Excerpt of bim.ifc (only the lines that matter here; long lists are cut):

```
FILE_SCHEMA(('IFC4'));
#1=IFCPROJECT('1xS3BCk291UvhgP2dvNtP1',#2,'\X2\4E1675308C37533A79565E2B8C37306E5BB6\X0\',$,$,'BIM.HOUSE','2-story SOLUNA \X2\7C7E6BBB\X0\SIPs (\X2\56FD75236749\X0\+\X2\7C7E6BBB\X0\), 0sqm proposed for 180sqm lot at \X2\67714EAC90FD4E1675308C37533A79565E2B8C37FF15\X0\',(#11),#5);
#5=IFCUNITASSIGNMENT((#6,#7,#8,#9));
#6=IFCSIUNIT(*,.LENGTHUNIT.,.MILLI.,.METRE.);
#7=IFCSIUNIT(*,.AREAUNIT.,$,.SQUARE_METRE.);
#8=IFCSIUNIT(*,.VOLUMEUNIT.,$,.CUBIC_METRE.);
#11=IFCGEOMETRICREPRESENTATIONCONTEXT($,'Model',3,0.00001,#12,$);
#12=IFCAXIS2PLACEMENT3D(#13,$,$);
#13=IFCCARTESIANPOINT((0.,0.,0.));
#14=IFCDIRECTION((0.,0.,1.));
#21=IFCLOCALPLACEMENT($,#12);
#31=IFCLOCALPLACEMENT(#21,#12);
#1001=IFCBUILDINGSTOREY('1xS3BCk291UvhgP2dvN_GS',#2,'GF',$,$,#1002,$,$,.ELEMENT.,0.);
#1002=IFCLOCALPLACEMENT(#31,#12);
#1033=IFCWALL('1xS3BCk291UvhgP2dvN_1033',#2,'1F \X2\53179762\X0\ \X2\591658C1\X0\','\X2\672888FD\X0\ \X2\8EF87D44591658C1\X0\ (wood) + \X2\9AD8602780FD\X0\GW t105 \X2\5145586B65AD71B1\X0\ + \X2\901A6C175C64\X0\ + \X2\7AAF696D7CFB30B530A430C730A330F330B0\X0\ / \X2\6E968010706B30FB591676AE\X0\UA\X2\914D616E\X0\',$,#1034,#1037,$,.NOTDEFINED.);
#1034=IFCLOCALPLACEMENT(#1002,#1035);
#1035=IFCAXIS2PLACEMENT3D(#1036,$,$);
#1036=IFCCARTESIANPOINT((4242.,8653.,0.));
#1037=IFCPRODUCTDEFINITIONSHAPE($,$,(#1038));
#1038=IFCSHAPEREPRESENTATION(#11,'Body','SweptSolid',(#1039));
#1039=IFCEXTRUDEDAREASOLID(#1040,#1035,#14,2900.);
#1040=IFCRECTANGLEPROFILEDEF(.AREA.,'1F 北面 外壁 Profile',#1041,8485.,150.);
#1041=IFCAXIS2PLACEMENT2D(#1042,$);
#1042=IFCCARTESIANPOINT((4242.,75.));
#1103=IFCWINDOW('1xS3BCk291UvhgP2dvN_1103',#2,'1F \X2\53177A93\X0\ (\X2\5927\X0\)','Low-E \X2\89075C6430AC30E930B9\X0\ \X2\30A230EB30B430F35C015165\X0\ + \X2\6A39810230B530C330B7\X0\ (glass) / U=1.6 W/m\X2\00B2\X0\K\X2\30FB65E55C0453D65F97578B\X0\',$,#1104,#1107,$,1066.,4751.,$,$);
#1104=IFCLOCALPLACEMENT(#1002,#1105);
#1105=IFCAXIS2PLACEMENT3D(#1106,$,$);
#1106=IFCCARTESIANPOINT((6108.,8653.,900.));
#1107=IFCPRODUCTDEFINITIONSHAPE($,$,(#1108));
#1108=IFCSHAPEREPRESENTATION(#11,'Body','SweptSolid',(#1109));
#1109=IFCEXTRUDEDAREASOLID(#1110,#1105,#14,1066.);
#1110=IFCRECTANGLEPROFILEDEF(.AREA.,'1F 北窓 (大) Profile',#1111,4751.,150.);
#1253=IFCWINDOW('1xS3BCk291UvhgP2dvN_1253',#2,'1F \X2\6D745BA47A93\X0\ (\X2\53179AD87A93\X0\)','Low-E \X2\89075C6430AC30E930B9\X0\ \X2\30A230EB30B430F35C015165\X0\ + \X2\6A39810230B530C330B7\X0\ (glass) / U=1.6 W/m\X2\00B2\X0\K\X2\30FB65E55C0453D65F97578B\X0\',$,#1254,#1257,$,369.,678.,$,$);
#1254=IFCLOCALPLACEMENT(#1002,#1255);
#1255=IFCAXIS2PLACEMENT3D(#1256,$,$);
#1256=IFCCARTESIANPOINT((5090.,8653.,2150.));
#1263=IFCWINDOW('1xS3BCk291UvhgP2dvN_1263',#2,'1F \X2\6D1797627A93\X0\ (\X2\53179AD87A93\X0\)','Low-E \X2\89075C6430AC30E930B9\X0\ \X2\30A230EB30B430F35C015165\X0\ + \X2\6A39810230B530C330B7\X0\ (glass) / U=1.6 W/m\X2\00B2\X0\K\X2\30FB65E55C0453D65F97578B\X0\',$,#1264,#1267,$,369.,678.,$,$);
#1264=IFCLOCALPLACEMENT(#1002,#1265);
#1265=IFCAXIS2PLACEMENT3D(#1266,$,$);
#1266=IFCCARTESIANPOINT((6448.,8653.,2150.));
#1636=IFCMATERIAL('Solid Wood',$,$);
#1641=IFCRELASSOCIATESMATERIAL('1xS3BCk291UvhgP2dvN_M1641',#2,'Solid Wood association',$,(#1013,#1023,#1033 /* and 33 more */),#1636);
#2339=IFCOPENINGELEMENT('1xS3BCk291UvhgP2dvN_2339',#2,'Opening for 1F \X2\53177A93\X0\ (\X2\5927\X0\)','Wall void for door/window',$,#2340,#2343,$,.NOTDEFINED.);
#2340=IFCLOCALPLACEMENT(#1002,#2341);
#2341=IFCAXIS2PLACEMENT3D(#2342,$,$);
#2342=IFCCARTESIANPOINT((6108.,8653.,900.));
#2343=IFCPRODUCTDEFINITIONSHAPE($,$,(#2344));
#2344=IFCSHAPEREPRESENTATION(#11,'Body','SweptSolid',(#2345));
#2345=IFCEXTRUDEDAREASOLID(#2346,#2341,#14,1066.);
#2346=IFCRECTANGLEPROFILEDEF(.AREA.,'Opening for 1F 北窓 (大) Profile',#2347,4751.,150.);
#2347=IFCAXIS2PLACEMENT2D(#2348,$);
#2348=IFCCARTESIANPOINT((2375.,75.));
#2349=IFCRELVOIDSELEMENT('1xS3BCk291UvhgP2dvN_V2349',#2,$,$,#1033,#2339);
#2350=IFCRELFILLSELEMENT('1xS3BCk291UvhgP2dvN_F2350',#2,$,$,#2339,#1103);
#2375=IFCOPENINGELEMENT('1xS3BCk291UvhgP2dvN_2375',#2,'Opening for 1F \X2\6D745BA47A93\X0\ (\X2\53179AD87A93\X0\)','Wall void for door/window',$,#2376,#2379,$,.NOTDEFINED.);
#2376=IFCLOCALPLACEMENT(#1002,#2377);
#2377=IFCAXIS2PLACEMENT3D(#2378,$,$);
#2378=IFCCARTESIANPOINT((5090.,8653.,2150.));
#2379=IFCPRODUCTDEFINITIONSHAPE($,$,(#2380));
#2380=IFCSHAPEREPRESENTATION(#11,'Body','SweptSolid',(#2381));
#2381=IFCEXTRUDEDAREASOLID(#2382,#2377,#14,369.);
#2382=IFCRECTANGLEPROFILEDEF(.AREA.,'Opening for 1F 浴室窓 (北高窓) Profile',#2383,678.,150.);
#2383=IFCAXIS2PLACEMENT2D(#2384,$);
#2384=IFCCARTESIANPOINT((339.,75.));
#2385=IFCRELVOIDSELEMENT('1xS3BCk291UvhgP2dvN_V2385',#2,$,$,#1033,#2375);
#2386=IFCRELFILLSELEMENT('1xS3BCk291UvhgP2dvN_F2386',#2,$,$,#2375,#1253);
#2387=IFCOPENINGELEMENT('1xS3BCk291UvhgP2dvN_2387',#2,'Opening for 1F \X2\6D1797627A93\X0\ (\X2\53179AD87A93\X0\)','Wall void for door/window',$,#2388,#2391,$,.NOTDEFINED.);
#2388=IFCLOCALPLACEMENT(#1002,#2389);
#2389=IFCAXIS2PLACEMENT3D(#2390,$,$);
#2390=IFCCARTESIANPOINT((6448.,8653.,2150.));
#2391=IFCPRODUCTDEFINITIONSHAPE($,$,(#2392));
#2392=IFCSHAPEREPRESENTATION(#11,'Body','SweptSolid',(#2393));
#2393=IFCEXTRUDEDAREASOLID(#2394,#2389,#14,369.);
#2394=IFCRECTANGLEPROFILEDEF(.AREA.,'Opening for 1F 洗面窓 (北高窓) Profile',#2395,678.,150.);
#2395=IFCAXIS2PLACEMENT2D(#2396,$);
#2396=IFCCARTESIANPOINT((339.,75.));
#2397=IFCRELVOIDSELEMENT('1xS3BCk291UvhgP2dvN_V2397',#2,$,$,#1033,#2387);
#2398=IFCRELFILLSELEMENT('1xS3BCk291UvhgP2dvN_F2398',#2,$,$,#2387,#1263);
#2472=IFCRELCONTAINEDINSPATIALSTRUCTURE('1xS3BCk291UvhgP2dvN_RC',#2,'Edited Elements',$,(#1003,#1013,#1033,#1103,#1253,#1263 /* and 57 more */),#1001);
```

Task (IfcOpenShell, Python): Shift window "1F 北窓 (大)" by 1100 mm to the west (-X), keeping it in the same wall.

```python
import ifcopenshell
import ifcopenshell.api.geometry
import ifcopenshell.util.placement
import ifcopenshell.util.unit

model = ifcopenshell.open("bim.ifc")
unit_scale = ifcopenshell.util.unit.calculate_unit_scale(model)

window = model.by_id(1103)
opening = window.FillsVoids[0].RelatingOpeningElement
wall = opening.VoidsElements[0].RelatingBuildingElement

wall_matrix = ifcopenshell.util.placement.get_local_placement(wall.ObjectPlacement)
shift = wall_matrix[:3, 0] * -1.1 / unit_scale
before = ifcopenshell.util.placement.get_local_placement(window.ObjectPlacement)[:3, 3].copy()

# The window is not placed relative to its opening, so move both.
for product in (opening, window):
    matrix = ifcopenshell.util.placement.get_local_placement(product.ObjectPlacement)
    matrix[:3, 3] += shift
    ifcopenshell.api.geometry.edit_object_placement(model, product=product, matrix=matrix, is_si=False)

after = ifcopenshell.util.placement.get_local_placement(window.ObjectPlacement)[:3, 3]
print("window moved by", (after - before).round(3) + 0.0)

model.write("bim-out.ifc")
```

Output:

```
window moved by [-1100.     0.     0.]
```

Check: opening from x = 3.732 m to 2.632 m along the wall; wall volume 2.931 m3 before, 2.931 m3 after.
